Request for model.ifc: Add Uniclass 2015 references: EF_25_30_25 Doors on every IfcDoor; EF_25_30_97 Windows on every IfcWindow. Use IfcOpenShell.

First a look at what the model holds.

```python
import ifcopenshell

model = ifcopenshell.open("model.ifc")
print(model.schema)
print("classifications:", [c.Name for c in model.by_type("IfcClassification")])
for ifc_class in ("IfcDoor", "IfcRoof", "IfcStair", "IfcWall", "IfcWindow"):
    print(ifc_class, len(model.by_type(ifc_class)))
```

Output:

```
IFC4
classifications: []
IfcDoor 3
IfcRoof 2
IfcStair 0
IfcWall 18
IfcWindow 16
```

```python
import ifcopenshell
import ifcopenshell.api.classification

model = ifcopenshell.open("model.ifc")

system = ifcopenshell.api.classification.add_classification(model, classification="Uniclass 2015")

codes = {
    "IfcDoor": ("EF_25_30_25", "Doors"),
    "IfcWindow": ("EF_25_30_97", "Windows"),
}
for ifc_class, (code, name) in codes.items():
    products = model.by_type(ifc_class)
    ifcopenshell.api.classification.add_reference(
        model, products=products, classification=system, identification=code, name=name
    )
    print(code, len(products))

model.write("model_rev.ifc")
```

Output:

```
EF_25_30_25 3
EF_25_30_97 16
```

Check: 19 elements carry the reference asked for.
